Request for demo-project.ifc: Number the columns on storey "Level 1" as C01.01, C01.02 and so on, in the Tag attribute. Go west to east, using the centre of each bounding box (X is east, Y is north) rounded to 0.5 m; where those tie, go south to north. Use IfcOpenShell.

First a look at what the model holds.

```python
import ifcopenshell
import ifcopenshell.util.element
import ifcopenshell.util.placement

model = ifcopenshell.open("demo-project.ifc")
print(model.schema)
storey = next(s for s in model.by_type("IfcBuildingStorey") if s.Name == "Level 1")
columns = [e for e in ifcopenshell.util.element.get_decomposition(storey) if e.is_a("IfcColumn")]
for e in sorted(columns, key=lambda e: e.id()):
    origin = ifcopenshell.util.placement.get_local_placement(e.ObjectPlacement)[:3, 3]
    print(e.id(), e.Tag, e.Name, origin.round(2) + 0.0, sep=" | ")
```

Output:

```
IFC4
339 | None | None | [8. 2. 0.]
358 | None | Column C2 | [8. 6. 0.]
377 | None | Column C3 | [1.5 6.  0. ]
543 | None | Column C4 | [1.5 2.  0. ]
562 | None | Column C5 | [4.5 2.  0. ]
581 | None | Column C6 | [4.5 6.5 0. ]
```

```python
import ifcopenshell
import ifcopenshell.geom
import ifcopenshell.util.element
import ifcopenshell.util.shape

model = ifcopenshell.open("demo-project.ifc")
settings = ifcopenshell.geom.settings()
settings.set("use-world-coords", True)


def centre(element):
    shape = ifcopenshell.geom.create_shape(settings, element)
    return ifcopenshell.util.shape.get_bbox_centroid(shape.geometry)


storey = next(s for s in model.by_type("IfcBuildingStorey") if s.Name == "Level 1")
columns = [e for e in ifcopenshell.util.element.get_decomposition(storey) if e.is_a("IfcColumn")]

# Insertion points can sit at a corner or the storey origin, so sort by the geometry (in metres).
centres = {e: centre(e) for e in columns}
columns.sort(key=lambda e: (round(centres[e][0] / 0.5), centres[e][1]))

for i, e in enumerate(columns, start=1):
    number = f"C01.{i:02d}"
    e.Tag = number
    print(e.id(), number)

model.write("demo-project-out.ifc")
```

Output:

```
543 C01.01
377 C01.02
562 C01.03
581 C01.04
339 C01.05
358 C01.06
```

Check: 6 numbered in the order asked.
